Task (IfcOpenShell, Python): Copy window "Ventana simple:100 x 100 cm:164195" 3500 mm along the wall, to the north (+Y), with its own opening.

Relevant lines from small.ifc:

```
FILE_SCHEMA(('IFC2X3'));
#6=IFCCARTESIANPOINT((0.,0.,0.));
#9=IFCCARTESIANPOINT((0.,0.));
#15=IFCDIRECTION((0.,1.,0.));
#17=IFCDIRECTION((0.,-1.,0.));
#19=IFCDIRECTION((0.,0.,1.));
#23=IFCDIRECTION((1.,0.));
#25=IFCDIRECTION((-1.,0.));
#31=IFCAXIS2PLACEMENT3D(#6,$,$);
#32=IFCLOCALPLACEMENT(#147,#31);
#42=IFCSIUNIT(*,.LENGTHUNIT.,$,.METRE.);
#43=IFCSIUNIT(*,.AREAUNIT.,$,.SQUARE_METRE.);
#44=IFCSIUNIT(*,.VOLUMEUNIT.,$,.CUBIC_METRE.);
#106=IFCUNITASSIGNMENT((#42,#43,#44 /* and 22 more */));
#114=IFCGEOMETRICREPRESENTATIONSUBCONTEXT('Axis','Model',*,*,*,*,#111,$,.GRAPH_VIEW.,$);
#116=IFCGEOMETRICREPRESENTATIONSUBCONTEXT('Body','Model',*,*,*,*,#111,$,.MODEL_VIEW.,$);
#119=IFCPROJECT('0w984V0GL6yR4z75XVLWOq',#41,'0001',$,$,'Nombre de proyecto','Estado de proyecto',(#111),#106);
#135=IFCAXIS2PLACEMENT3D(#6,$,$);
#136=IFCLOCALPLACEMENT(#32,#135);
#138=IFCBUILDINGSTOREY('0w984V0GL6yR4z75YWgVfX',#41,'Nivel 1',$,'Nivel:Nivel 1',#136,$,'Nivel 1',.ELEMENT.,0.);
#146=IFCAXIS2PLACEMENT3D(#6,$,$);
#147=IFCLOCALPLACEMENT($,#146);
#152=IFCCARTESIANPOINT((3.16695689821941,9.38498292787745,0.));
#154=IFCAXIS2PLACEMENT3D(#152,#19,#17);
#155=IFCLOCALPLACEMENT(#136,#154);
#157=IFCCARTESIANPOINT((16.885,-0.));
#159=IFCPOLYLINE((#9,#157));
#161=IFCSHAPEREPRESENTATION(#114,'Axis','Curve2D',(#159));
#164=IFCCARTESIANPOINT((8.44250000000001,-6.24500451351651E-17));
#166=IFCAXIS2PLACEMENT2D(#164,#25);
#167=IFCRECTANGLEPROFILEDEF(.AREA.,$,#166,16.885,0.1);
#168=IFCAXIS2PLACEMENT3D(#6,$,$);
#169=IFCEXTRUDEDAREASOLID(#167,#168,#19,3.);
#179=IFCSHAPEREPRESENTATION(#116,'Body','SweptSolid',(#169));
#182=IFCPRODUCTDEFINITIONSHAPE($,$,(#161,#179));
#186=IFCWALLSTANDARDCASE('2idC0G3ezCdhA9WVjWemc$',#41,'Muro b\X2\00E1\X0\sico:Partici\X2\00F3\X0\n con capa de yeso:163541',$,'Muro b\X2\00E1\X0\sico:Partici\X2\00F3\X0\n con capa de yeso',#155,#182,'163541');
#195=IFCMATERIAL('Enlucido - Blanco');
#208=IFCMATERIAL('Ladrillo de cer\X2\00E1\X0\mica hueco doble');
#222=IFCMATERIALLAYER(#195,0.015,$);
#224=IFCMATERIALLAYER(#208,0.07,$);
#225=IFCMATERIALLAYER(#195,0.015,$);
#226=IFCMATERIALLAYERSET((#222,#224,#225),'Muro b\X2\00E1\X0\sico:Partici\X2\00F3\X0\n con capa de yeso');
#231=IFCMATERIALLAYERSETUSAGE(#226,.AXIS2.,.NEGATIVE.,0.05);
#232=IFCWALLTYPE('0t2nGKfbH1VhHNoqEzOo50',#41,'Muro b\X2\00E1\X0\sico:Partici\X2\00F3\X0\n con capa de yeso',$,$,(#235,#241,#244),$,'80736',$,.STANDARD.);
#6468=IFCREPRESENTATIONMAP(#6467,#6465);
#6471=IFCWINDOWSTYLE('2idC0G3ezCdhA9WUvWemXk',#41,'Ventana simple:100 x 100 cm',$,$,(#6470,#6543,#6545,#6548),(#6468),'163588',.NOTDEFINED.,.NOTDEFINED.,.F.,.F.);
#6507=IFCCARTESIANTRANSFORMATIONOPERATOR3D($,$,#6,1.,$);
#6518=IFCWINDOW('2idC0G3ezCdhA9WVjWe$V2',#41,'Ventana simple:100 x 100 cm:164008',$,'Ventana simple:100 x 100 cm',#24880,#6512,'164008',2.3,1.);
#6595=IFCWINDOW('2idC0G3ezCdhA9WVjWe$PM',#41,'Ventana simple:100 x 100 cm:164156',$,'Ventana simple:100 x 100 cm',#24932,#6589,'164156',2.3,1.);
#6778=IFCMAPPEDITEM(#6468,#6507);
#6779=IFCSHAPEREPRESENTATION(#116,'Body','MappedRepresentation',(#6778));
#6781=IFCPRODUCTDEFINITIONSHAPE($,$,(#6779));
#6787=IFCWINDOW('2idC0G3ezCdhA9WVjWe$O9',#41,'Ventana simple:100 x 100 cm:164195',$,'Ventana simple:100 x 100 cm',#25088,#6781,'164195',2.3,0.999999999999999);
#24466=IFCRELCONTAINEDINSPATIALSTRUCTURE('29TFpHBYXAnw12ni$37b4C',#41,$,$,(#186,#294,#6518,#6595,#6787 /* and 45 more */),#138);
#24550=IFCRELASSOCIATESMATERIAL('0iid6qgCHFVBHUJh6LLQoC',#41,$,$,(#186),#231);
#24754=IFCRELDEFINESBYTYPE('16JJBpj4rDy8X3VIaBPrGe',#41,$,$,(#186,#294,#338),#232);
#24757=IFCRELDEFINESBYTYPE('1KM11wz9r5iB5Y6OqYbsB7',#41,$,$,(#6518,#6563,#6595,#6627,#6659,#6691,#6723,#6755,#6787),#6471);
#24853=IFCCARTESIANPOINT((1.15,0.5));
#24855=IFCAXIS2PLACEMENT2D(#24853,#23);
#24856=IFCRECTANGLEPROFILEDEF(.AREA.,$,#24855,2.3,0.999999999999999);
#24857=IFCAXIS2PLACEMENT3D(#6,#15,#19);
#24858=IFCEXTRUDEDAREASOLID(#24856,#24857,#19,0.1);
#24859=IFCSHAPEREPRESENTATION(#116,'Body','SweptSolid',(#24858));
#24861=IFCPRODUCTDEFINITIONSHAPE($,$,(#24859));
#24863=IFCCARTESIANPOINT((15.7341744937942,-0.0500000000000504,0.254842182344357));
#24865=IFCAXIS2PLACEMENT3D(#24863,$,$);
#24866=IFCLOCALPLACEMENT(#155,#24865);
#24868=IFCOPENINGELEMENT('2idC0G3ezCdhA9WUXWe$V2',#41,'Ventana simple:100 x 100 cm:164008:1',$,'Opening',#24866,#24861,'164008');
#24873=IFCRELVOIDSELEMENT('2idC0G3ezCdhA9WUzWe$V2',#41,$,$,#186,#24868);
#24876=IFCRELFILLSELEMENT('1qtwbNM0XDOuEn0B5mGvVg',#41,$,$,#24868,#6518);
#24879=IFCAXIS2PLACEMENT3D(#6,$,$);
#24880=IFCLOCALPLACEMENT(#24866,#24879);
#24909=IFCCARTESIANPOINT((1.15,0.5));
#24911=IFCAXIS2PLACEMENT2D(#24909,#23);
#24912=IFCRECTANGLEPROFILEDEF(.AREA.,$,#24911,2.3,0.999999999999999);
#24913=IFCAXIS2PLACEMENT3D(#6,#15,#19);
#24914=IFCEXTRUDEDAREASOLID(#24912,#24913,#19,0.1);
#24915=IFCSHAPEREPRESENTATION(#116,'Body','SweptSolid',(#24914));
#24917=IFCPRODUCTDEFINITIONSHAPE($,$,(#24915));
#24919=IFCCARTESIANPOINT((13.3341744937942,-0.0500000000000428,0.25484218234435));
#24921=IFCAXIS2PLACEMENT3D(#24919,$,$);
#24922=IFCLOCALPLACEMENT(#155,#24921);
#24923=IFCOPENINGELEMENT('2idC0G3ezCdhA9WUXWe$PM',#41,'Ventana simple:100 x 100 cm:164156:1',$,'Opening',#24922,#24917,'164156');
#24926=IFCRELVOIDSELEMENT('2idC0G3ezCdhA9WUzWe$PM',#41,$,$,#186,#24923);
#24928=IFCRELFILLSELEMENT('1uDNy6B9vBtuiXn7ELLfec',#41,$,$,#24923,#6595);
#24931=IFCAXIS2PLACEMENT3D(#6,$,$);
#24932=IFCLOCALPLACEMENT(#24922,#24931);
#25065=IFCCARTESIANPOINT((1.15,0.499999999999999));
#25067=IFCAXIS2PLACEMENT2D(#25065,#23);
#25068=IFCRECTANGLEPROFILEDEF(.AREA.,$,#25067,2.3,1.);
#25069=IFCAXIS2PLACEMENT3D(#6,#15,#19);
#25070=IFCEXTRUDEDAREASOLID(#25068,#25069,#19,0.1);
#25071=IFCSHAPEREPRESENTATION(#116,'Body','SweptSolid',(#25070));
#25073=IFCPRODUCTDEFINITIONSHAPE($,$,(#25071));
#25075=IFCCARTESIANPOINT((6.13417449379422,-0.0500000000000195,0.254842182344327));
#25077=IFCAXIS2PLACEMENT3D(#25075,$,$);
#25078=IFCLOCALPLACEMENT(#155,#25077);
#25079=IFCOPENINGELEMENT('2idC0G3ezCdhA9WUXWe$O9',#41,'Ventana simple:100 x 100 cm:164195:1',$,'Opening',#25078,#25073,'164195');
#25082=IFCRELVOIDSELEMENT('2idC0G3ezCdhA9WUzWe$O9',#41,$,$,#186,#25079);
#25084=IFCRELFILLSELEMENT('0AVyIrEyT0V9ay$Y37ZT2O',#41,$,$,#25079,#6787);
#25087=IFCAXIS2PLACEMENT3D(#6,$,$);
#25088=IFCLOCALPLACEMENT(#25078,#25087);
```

```python
import ifcopenshell
import ifcopenshell.api.feature
import ifcopenshell.api.geometry
import ifcopenshell.api.root
import ifcopenshell.geom
import ifcopenshell.util.element
import ifcopenshell.util.placement
import ifcopenshell.util.shape
import ifcopenshell.util.unit

model = ifcopenshell.open("small.ifc")
unit_scale = ifcopenshell.util.unit.calculate_unit_scale(model)
settings = ifcopenshell.geom.settings()


def volume(element):
    """Net volume in cubic metres, openings subtracted."""
    shape = ifcopenshell.geom.create_shape(settings, element)
    return ifcopenshell.util.shape.get_volume(shape.geometry)


def reuse_history(source, copy):
    """copy_class also copies each property set's owner history, people and application; keep the originals."""
    for rel in copy.IsDefinedBy:
        if rel.is_a("IfcRelDefinesByProperties") and (history := rel.RelatingPropertyDefinition.OwnerHistory):
            rel.RelatingPropertyDefinition.OwnerHistory = source.OwnerHistory
            ifcopenshell.util.element.remove_deep2(model, history)


window = model.by_guid("2idC0G3ezCdhA9WVjWe$O9")
opening = window.FillsVoids[0].RelatingOpeningElement
wall = opening.VoidsElements[0].RelatingBuildingElement
before = volume(wall)
shift = ifcopenshell.util.placement.get_local_placement(wall.ObjectPlacement)[:3, 0] * -3.5 / unit_scale

# copy_class copies the void relationship, type, container and properties, but no geometry.
new_opening = ifcopenshell.api.root.copy_class(model, product=opening)
new_opening.Representation = ifcopenshell.util.element.copy_deep(
    model, opening.Representation, exclude=["IfcGeometricRepresentationContext", "IfcRepresentationMap"]
)
new_opening.Name = "Ventana simple:100 x 100 cm"
new_opening.Tag = None
new_window = ifcopenshell.api.root.copy_class(model, product=window)
new_window.Representation = ifcopenshell.util.element.copy_deep(
    model, window.Representation, exclude=["IfcGeometricRepresentationContext", "IfcRepresentationMap"]
)
new_window.Name = "Ventana simple:100 x 100 cm"
new_window.Tag = None
reuse_history(window, new_window)
fills = ifcopenshell.api.feature.add_filling(model, opening=new_opening, element=new_window)
fills.OwnerHistory = new_window.OwnerHistory  # required in IFC2X3

for old, new in ((opening, new_opening), (window, new_window)):
    matrix = ifcopenshell.util.placement.get_local_placement(old.ObjectPlacement)
    matrix[:3, 3] += shift
    ifcopenshell.api.geometry.edit_object_placement(model, product=new, matrix=matrix, is_si=False)

after = volume(wall)

print(f"wall volume {before:.3f} -> {after:.3f} m3")

model.write("small-out.ifc")
```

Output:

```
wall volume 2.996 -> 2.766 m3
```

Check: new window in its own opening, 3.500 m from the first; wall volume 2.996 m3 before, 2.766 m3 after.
